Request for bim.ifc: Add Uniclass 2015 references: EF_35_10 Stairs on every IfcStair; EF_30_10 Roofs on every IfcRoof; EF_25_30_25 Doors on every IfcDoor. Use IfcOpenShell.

First a look at what the model holds.

```python
import ifcopenshell

model = ifcopenshell.open("bim.ifc")
print(model.schema)
print("classifications:", [c.Name for c in model.by_type("IfcClassification")])
for ifc_class in ("IfcDoor", "IfcRoof", "IfcStair", "IfcWall", "IfcWindow"):
    print(ifc_class, len(model.by_type(ifc_class)))
```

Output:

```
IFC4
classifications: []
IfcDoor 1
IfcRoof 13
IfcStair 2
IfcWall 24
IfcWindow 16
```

```python
import ifcopenshell
import ifcopenshell.api.classification

model = ifcopenshell.open("bim.ifc")

system = ifcopenshell.api.classification.add_classification(model, classification="Uniclass 2015")

codes = {
    "IfcStair": ("EF_35_10", "Stairs"),
    "IfcRoof": ("EF_30_10", "Roofs"),
    "IfcDoor": ("EF_25_30_25", "Doors"),
}
for ifc_class, (code, name) in codes.items():
    products = model.by_type(ifc_class)
    ifcopenshell.api.classification.add_reference(
        model, products=products, classification=system, identification=code, name=name
    )
    print(code, len(products))

model.write("bim_rev.ifc")
```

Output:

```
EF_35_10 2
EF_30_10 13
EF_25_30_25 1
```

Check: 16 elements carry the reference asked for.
